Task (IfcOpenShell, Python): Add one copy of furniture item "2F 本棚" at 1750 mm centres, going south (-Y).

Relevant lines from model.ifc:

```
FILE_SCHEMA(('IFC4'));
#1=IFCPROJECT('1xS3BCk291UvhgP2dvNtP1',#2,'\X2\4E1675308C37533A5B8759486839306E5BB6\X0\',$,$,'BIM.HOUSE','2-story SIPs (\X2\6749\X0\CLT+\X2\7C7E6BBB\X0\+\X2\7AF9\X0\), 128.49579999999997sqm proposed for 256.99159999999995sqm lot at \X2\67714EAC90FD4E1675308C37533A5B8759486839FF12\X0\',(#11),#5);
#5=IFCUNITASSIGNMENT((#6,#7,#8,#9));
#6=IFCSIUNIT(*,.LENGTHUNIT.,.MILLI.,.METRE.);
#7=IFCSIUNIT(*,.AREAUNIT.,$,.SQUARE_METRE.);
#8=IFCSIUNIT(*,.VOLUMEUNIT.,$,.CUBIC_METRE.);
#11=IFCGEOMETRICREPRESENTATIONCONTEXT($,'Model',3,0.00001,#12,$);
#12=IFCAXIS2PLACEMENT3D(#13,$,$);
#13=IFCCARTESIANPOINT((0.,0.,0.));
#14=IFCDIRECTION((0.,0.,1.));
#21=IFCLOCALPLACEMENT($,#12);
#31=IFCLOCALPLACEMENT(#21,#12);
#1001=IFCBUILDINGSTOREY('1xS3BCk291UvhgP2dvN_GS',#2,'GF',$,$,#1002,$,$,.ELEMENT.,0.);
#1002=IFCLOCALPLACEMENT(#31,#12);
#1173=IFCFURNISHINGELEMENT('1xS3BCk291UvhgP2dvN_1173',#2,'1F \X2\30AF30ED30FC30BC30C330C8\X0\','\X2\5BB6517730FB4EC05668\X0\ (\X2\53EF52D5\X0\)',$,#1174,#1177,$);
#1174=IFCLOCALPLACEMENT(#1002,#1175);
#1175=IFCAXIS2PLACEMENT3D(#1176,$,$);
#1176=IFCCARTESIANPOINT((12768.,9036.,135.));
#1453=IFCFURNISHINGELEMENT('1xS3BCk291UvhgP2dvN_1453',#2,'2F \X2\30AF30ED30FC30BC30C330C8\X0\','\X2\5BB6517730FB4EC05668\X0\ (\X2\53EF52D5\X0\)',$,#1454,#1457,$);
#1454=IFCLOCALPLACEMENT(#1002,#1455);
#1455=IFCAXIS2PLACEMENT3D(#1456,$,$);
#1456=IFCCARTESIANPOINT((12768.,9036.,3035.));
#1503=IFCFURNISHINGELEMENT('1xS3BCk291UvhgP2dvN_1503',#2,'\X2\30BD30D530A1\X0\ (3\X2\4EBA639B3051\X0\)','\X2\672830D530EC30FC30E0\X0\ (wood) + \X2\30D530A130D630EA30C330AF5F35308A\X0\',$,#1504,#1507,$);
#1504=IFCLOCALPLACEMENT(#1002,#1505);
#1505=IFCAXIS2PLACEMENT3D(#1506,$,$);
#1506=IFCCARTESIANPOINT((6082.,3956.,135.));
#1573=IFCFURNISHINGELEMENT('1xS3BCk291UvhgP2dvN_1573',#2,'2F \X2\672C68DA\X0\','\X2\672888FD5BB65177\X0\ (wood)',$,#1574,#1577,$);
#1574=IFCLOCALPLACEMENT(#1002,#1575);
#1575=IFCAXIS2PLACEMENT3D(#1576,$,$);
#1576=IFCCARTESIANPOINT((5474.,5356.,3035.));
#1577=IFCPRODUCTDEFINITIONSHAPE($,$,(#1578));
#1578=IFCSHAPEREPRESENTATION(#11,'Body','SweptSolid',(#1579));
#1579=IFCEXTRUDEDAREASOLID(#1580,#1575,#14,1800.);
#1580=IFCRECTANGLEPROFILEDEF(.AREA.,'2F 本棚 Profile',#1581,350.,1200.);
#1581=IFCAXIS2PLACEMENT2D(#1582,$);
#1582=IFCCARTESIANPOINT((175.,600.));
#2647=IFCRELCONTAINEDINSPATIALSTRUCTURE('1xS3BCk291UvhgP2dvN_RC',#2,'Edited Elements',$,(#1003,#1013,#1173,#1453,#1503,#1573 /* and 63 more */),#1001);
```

```python
import numpy as np
import ifcopenshell
import ifcopenshell.api.geometry
import ifcopenshell.api.root
import ifcopenshell.util.element
import ifcopenshell.util.placement

model = ifcopenshell.open("model.ifc")


def reuse_history(source, copy):
    """copy_class also copies each property set's owner history, people and application; keep the originals."""
    for rel in copy.IsDefinedBy:
        if rel.is_a("IfcRelDefinesByProperties") and (history := rel.RelatingPropertyDefinition.OwnerHistory):
            rel.RelatingPropertyDefinition.OwnerHistory = source.OwnerHistory
            ifcopenshell.util.element.remove_deep2(model, history)


source = model.by_id(1573)
base = ifcopenshell.util.placement.get_local_placement(source.ObjectPlacement)
step = np.array([0.0, -1.0, 0.0]) * 1750.0

for i in range(1, 2):
    copy = ifcopenshell.api.root.copy_class(model, product=source)
    copy.Representation = ifcopenshell.util.element.copy_deep(
        model, source.Representation, exclude=["IfcGeometricRepresentationContext", "IfcRepresentationMap"]
    )
    reuse_history(source, copy)
    matrix = base.copy()
    matrix[:3, 3] += i * step
    print("added at", matrix[:3, 3].round(3) + 0.0)
    ifcopenshell.api.geometry.edit_object_placement(model, product=copy, matrix=matrix, is_si=False)

model.write("model_v2.ifc")
```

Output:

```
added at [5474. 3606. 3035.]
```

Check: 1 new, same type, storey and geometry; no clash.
